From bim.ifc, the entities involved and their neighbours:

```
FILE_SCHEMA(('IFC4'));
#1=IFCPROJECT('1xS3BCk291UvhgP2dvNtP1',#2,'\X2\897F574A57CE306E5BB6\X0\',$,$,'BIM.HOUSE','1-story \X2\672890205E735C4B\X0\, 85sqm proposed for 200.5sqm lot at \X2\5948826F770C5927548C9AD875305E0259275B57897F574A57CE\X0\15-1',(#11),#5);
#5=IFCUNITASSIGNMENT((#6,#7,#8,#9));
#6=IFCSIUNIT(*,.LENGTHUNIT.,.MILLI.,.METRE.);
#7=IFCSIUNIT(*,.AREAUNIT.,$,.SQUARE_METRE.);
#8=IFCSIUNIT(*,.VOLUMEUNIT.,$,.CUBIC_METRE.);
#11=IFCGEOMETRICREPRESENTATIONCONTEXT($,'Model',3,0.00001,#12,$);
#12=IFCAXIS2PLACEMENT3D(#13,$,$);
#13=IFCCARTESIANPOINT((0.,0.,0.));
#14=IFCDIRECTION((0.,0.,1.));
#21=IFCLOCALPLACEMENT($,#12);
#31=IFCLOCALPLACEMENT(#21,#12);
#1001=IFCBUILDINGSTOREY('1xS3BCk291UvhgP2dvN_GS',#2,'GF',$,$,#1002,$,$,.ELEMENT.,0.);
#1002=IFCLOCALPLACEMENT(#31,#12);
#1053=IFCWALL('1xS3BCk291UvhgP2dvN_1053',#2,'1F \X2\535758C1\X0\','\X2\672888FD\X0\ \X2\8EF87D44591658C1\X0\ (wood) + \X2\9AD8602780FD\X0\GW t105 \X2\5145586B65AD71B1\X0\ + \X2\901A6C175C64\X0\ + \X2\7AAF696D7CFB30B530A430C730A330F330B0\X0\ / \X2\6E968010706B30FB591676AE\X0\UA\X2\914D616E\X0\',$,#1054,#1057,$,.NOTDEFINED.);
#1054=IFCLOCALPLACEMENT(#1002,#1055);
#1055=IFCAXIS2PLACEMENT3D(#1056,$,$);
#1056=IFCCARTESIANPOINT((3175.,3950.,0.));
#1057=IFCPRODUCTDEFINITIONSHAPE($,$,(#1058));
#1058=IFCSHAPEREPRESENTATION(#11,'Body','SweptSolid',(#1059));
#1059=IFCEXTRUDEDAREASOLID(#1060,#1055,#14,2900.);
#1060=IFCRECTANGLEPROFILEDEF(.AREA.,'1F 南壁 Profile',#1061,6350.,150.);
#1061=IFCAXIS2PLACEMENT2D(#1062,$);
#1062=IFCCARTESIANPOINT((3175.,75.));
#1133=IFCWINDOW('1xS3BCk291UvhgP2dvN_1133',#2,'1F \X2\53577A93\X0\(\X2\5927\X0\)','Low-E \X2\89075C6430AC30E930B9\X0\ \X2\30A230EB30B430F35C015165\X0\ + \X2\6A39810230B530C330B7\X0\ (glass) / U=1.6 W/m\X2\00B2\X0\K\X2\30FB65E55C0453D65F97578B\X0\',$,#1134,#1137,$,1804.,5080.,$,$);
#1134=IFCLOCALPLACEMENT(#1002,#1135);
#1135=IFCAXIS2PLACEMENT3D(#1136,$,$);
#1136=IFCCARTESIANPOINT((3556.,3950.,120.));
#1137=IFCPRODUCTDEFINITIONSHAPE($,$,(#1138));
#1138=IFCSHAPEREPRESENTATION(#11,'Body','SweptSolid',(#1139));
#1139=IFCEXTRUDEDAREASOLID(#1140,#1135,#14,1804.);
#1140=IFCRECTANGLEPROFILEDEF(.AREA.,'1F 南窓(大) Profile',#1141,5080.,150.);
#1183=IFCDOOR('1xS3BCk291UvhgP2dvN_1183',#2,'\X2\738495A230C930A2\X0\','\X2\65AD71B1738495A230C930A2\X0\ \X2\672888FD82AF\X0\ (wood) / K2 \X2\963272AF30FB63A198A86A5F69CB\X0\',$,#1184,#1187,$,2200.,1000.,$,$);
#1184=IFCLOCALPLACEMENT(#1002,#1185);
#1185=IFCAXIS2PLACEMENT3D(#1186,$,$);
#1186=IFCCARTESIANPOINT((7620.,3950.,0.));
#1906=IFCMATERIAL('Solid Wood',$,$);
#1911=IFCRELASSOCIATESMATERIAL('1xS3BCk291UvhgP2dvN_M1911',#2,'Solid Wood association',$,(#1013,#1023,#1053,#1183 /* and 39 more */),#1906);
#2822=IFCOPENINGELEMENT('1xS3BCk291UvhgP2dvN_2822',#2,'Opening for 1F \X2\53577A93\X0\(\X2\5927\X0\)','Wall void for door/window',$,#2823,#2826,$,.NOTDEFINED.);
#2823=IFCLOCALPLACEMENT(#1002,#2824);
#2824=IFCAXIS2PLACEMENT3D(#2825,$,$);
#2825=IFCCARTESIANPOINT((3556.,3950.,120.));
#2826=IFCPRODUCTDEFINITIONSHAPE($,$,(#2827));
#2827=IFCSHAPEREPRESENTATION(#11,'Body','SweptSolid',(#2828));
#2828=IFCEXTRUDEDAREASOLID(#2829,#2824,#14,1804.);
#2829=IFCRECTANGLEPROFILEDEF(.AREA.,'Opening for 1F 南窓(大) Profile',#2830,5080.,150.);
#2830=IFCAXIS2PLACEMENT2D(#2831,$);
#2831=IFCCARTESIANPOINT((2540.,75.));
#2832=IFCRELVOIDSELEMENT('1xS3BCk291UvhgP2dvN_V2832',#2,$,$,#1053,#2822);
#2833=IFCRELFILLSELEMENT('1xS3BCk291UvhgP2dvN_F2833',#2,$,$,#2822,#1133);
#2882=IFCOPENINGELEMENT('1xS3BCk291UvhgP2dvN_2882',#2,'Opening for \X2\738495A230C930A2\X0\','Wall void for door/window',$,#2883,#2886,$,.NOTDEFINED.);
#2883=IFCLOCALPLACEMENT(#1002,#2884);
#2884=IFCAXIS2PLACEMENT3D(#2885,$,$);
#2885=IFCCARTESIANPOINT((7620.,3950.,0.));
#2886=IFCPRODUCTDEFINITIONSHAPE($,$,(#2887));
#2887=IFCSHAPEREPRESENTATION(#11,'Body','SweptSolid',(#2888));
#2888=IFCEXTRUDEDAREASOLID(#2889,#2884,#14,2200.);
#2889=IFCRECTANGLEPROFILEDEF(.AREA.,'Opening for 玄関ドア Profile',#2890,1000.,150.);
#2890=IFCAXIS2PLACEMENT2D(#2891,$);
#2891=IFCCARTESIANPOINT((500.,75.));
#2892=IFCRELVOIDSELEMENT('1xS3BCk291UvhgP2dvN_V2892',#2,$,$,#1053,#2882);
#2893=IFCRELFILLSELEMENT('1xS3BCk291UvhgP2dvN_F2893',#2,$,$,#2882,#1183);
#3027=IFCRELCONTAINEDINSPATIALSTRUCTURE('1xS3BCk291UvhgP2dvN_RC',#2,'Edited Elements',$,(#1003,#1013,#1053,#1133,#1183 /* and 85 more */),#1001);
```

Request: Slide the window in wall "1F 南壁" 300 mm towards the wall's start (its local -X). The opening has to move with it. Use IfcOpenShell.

```python
import ifcopenshell
import ifcopenshell.api.geometry
import ifcopenshell.util.placement

model = ifcopenshell.open("bim.ifc")

window = model.by_id(1133)
opening = window.FillsVoids[0].RelatingOpeningElement
wall = opening.VoidsElements[0].RelatingBuildingElement

wall_matrix = ifcopenshell.util.placement.get_local_placement(wall.ObjectPlacement)
shift = wall_matrix[:3, 0] * -300.0
before = ifcopenshell.util.placement.get_local_placement(window.ObjectPlacement)[:3, 3].copy()

# The window is not placed relative to its opening, so move both.
for product in (opening, window):
    matrix = ifcopenshell.util.placement.get_local_placement(product.ObjectPlacement)
    matrix[:3, 3] += shift
    ifcopenshell.api.geometry.edit_object_placement(model, product=product, matrix=matrix, is_si=False)

after = ifcopenshell.util.placement.get_local_placement(window.ObjectPlacement)[:3, 3]
print("window moved by", (after - before).round(3) + 0.0)

model.write("bim_updated.ifc")
```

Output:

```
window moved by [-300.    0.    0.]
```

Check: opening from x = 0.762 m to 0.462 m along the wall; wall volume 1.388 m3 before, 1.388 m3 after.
